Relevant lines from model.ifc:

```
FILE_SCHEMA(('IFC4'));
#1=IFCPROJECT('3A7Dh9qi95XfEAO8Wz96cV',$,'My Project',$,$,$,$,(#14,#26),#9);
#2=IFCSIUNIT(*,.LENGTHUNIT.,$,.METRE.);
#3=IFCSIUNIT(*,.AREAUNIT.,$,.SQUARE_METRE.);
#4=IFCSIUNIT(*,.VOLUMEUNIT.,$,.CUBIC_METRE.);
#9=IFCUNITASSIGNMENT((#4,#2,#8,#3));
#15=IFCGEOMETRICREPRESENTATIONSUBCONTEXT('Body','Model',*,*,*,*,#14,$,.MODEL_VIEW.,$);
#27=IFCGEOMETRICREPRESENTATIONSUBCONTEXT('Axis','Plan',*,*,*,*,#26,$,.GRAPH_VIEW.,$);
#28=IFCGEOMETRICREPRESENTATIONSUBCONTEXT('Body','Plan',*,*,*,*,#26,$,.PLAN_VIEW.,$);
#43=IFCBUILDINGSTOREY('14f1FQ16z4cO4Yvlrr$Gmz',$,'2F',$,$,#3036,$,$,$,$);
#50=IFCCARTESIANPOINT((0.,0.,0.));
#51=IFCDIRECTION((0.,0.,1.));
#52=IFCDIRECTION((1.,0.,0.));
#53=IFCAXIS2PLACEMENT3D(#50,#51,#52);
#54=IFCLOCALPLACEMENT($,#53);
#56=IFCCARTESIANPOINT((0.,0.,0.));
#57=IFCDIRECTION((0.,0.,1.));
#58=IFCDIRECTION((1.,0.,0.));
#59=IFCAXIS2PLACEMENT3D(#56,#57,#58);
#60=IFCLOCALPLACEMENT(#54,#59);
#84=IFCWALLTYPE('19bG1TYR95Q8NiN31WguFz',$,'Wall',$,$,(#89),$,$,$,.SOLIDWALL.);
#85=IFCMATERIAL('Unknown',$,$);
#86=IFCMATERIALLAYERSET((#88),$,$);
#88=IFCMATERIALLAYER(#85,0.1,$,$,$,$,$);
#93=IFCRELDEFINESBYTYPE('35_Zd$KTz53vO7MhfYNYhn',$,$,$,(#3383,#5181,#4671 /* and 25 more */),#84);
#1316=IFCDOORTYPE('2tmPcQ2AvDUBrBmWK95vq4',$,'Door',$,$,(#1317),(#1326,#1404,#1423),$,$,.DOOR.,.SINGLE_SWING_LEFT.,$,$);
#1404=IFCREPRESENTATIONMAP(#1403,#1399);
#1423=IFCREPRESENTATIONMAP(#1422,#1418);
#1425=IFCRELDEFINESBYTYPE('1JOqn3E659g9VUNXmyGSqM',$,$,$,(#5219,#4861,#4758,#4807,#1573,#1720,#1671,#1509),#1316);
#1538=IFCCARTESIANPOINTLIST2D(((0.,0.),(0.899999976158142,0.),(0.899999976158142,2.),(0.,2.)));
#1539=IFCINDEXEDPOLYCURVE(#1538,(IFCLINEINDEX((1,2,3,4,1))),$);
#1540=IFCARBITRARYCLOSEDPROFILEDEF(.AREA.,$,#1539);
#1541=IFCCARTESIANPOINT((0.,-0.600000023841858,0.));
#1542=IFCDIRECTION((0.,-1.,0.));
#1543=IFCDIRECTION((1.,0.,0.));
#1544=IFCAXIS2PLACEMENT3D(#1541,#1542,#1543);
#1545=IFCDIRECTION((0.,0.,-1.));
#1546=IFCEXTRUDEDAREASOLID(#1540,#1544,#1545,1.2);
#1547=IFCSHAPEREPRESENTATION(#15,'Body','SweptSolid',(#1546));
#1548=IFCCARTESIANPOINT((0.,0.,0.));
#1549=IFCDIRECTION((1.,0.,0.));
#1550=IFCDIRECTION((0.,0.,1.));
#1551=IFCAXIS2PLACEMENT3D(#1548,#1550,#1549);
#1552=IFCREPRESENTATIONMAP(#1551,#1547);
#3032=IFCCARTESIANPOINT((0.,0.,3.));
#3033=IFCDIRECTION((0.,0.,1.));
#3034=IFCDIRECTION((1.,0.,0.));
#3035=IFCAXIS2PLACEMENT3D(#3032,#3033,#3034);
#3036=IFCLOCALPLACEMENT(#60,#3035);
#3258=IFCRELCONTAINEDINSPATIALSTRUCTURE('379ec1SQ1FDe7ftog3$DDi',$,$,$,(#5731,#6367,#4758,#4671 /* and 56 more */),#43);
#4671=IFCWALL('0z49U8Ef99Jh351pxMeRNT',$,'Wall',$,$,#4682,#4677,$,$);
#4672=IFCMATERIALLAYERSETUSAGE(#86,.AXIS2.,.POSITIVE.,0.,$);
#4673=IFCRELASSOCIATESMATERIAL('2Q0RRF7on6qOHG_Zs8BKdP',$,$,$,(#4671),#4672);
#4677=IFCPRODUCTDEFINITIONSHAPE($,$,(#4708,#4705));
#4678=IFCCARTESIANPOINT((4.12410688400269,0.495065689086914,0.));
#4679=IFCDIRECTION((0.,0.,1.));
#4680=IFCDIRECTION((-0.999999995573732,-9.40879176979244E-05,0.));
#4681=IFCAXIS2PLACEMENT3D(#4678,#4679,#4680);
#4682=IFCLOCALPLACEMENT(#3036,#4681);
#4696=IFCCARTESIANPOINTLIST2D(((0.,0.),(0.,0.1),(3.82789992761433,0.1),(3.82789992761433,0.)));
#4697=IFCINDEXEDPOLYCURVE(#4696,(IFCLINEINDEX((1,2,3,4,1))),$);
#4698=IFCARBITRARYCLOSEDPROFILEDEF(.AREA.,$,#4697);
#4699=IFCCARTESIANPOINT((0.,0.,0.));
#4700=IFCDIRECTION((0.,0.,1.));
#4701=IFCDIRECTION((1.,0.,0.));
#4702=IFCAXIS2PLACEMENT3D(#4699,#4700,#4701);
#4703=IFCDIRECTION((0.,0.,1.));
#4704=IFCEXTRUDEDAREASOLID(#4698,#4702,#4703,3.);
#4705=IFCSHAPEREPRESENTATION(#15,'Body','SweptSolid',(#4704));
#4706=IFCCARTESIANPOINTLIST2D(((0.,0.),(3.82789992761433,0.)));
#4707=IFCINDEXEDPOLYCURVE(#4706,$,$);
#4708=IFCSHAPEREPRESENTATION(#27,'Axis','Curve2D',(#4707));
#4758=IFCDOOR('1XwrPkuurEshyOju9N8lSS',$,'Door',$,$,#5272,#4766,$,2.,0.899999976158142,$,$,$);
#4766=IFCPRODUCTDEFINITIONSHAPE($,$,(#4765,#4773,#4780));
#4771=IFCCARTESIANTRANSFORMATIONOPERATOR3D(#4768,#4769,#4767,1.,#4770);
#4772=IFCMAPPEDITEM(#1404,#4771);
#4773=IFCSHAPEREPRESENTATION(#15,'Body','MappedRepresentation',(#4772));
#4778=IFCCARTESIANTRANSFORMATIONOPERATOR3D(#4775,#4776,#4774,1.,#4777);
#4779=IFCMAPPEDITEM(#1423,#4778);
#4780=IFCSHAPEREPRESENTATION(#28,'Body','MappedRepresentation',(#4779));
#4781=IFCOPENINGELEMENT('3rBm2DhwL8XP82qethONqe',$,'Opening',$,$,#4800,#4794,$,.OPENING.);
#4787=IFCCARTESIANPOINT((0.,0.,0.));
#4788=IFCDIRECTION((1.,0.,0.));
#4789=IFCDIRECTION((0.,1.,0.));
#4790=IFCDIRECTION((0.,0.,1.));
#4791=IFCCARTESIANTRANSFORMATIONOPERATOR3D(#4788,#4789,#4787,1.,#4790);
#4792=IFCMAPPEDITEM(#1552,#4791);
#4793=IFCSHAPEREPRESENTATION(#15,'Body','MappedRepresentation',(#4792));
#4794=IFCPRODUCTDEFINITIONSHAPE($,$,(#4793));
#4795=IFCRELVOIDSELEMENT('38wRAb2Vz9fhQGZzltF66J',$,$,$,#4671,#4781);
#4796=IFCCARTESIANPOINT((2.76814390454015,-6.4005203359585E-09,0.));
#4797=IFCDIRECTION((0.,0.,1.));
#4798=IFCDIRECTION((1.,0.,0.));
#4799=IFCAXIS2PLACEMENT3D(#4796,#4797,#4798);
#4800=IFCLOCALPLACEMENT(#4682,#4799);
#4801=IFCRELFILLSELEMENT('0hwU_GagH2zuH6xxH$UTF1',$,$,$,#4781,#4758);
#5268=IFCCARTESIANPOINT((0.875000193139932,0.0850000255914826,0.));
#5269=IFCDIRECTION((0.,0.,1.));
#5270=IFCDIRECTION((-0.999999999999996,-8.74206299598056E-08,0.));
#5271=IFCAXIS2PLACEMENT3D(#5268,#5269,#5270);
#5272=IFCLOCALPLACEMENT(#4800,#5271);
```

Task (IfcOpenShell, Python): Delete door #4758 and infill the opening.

```python
import ifcopenshell
import ifcopenshell.api.feature
import ifcopenshell.api.root
import ifcopenshell.geom
import ifcopenshell.util.shape

model = ifcopenshell.open("model.ifc")
settings = ifcopenshell.geom.settings()


def volume(element):
    """Net volume in cubic metres, openings subtracted."""
    shape = ifcopenshell.geom.create_shape(settings, element)
    return ifcopenshell.util.shape.get_volume(shape.geometry)


door = model.by_guid("1XwrPkuurEshyOju9N8lSS")
opening = door.FillsVoids[0].RelatingOpeningElement
wall = opening.VoidsElements[0].RelatingBuildingElement
before = volume(wall)

ifcopenshell.api.root.remove_product(model, product=door)
ifcopenshell.api.feature.remove_feature(model, feature=opening)

after = volume(wall)

print(f"wall volume {before:.3f} -> {after:.3f} m3")

model.write("model_edited.ifc")
```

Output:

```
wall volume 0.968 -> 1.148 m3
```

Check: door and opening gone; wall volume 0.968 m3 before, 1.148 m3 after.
